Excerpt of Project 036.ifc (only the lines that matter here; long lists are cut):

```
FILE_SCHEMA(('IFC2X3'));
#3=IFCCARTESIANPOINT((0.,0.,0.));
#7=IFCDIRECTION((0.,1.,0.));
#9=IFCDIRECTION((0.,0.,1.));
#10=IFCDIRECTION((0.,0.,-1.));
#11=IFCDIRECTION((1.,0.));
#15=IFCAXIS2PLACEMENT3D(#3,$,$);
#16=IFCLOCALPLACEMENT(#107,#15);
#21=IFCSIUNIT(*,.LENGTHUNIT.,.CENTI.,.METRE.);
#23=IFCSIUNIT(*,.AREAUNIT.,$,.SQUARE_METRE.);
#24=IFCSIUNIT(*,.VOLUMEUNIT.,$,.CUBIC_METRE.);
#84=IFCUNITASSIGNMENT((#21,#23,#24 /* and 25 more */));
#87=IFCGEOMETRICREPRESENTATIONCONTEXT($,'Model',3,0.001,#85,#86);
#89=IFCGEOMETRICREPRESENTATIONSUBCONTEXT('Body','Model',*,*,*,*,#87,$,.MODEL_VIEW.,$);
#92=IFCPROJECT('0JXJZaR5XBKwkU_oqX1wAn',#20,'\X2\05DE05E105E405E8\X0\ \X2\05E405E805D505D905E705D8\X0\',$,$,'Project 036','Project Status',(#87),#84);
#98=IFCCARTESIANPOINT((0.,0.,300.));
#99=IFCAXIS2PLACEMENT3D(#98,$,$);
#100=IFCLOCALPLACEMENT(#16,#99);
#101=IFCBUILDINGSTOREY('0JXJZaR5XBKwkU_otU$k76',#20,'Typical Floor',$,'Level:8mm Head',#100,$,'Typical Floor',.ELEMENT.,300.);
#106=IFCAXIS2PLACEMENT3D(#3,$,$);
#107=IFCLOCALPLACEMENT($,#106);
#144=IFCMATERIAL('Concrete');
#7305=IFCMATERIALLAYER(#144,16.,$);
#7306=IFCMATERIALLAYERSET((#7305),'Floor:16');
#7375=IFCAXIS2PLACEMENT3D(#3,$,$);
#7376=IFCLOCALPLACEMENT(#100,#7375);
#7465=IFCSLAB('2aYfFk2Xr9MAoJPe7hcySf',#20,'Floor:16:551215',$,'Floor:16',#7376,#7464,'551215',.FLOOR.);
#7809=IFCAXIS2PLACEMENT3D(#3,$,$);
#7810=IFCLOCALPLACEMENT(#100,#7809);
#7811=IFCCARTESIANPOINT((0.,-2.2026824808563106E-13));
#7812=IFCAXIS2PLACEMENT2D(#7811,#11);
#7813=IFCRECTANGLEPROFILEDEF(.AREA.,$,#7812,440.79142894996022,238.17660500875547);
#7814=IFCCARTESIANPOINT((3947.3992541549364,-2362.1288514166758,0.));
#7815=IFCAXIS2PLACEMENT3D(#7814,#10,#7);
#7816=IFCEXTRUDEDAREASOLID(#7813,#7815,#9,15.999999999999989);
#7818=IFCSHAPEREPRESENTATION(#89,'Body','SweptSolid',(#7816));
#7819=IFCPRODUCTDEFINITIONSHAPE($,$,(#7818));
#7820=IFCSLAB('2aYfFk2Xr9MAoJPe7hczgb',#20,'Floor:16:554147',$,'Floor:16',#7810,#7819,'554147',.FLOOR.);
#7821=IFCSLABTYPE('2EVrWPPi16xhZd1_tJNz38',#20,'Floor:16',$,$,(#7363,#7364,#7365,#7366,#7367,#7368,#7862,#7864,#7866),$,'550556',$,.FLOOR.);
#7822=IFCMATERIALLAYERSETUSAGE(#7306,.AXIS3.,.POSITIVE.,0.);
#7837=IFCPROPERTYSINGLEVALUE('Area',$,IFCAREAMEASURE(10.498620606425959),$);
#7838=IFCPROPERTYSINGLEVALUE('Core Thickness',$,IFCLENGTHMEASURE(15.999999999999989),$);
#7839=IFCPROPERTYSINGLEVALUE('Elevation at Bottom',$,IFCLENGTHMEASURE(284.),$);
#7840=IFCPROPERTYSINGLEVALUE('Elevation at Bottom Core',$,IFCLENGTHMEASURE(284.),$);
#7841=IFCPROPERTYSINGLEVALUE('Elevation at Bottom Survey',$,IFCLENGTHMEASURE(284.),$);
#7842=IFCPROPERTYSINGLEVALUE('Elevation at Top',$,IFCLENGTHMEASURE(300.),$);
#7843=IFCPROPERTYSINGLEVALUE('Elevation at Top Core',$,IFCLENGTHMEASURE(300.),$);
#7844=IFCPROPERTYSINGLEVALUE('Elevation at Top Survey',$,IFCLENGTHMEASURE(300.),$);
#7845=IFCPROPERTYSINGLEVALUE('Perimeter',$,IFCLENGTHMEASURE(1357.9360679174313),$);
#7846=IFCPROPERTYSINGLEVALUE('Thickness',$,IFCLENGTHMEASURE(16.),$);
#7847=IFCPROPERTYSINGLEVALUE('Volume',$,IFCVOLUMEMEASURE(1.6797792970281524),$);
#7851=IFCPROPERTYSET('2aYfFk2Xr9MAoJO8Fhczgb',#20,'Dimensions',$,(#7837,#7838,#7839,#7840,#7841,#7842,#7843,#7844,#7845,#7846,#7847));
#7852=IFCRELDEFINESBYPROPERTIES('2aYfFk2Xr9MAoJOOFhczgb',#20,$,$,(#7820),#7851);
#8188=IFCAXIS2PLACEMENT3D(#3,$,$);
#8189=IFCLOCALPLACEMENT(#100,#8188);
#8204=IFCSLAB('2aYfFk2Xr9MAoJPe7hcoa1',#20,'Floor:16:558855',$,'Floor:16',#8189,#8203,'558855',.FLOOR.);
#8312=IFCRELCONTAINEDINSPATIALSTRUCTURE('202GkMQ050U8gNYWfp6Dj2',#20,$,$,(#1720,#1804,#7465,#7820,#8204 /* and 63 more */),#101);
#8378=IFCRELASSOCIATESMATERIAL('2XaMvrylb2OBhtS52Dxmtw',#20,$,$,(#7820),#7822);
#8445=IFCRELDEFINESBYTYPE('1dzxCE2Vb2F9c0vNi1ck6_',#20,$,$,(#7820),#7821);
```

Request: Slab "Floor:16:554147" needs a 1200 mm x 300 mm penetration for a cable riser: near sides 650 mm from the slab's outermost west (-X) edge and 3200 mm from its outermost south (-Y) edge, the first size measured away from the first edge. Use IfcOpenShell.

```python
import numpy as np
import ifcopenshell
import ifcopenshell.api.feature
import ifcopenshell.api.geometry
import ifcopenshell.api.pset
import ifcopenshell.api.root
import ifcopenshell.geom
import ifcopenshell.util.element
import ifcopenshell.util.placement
import ifcopenshell.util.representation
import ifcopenshell.util.shape
import ifcopenshell.util.unit

model = ifcopenshell.open("Project 036.ifc")
unit_scale = ifcopenshell.util.unit.calculate_unit_scale(model)
area_scale = ifcopenshell.util.unit.calculate_unit_scale(model, "AREAUNIT")
volume_scale = ifcopenshell.util.unit.calculate_unit_scale(model, "VOLUMEUNIT")
settings = ifcopenshell.geom.settings()


def volume(element):
    """Net volume in cubic metres, openings subtracted."""
    shape = ifcopenshell.geom.create_shape(settings, element)
    return ifcopenshell.util.shape.get_volume(shape.geometry)


slab = model.by_guid("2aYfFk2Xr9MAoJPe7hczgb")
before = volume(slab)

# Extent in the slab's own axes, in metres. The edges named are its -X and -Y sides.
slab_shape = ifcopenshell.geom.create_shape(settings, slab)
vertices = ifcopenshell.util.shape.get_vertices(slab_shape.geometry)
x_min, y_min, bottom = vertices.min(axis=0)
top = vertices[:, 2].max()

opening = ifcopenshell.api.root.create_entity(model, ifc_class="IfcOpeningElement", name="Cable riser opening")
context = ifcopenshell.util.representation.get_context(model, "Model", "Body", "MODEL_VIEW")
width, depth = 1.2, 0.3
outline = [(0.0, 0.0), (width, 0.0), (width, depth), (0.0, depth), (0.0, 0.0)]
# Overshoot both faces by 50 mm so the cut is clean.
shape = ifcopenshell.api.geometry.add_slab_representation(
    model, context=context, depth=top - bottom + 0.1, polyline=outline
)
ifcopenshell.api.geometry.assign_representation(model, product=opening, representation=shape)

matrix = ifcopenshell.util.placement.get_local_placement(slab.ObjectPlacement)
matrix[:, 3] = matrix @ np.append(np.array([x_min + 0.65, y_min + 3.2, bottom - 0.05]) / unit_scale, 1.0)
ifcopenshell.api.geometry.edit_object_placement(model, product=opening, matrix=matrix, is_si=False)
ifcopenshell.api.feature.add_feature(model, feature=opening, element=slab)

after = volume(slab)

# Update the slab's stored quantities.
pset = model.by_id(ifcopenshell.util.element.get_pset(slab, "Dimensions", should_inherit=False)["id"])
ifcopenshell.api.pset.edit_pset(model, pset=pset, properties={
    "Area": model.create_entity("IfcAreaMeasure", after / (top - bottom) / area_scale),
    "Volume": model.create_entity("IfcVolumeMeasure", after / volume_scale),
})

print(f"slab volume {before:.3f} -> {after:.3f} m3")

model.write("Project 036_v2.ifc")
```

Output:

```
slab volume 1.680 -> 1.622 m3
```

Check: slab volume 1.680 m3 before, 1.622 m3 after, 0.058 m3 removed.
